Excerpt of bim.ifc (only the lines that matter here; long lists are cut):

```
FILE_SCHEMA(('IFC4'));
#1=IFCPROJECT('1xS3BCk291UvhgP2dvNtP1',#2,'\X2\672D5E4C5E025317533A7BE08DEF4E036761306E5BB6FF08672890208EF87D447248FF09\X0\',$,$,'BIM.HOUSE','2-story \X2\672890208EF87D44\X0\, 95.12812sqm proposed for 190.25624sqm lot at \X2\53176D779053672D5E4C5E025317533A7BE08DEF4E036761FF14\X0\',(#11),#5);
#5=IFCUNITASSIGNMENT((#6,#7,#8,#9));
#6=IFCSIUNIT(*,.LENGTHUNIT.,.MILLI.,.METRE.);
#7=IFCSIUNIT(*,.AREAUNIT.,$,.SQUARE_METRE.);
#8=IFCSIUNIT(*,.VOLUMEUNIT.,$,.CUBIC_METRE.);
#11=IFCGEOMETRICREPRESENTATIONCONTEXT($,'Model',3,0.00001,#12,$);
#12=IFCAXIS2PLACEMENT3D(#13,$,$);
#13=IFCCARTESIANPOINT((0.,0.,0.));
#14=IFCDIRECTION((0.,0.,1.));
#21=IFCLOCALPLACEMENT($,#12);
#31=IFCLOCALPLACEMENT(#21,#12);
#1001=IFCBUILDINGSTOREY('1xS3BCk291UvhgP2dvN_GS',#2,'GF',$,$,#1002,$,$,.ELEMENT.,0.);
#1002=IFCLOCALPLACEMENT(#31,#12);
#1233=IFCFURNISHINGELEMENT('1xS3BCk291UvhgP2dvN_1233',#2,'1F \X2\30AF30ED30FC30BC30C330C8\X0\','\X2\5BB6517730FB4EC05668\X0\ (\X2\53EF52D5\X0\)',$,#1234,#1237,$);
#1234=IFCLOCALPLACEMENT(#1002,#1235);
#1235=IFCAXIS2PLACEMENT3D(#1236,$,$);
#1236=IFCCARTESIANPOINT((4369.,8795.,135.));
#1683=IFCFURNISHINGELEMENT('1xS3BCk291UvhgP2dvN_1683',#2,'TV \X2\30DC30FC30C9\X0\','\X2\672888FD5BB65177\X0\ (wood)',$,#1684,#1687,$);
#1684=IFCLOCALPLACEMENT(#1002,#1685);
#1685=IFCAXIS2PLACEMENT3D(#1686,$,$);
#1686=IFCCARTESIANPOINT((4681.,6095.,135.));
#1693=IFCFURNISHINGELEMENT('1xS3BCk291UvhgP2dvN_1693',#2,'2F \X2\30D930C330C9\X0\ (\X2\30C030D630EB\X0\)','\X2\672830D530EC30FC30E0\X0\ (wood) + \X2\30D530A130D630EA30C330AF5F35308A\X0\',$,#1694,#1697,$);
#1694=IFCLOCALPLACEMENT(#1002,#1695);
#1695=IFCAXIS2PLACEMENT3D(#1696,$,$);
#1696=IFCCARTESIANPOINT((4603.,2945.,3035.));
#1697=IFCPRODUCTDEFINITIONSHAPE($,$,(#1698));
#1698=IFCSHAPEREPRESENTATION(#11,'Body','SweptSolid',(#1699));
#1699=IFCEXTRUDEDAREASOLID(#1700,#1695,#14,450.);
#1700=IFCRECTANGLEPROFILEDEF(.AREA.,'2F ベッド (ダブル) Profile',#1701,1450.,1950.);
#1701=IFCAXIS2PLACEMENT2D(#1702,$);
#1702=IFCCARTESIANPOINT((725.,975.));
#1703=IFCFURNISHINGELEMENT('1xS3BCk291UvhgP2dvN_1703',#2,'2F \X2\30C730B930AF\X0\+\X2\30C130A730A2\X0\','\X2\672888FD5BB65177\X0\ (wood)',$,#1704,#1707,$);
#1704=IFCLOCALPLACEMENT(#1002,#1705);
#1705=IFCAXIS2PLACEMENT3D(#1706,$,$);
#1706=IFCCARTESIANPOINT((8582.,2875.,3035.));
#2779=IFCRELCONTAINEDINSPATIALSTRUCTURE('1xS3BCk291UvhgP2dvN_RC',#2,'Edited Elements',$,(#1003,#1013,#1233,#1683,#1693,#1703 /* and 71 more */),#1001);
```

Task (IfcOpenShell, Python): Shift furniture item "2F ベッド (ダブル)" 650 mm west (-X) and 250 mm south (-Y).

```python
import ifcopenshell
import ifcopenshell.api.geometry
import ifcopenshell.util.placement
import ifcopenshell.util.unit

model = ifcopenshell.open("bim.ifc")
unit_scale = ifcopenshell.util.unit.calculate_unit_scale(model)

item = model.by_guid("1xS3BCk291UvhgP2dvN_1693")
matrix = ifcopenshell.util.placement.get_local_placement(item.ObjectPlacement)
matrix[0, 3] -= 0.65 / unit_scale
matrix[1, 3] -= 0.25 / unit_scale
ifcopenshell.api.geometry.edit_object_placement(model, product=item, matrix=matrix, is_si=False)

print(ifcopenshell.util.placement.get_local_placement(item.ObjectPlacement).round(3) + 0.0)

model.write("bim_edited.ifc")
```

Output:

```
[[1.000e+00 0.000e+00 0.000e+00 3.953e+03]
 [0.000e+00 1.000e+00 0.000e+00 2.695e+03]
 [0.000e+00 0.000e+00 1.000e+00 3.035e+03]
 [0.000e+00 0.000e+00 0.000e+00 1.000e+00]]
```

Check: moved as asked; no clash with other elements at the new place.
